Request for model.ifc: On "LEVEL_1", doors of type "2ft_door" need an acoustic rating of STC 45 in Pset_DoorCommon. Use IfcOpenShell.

First a look at what the model holds.

```python
import ifcopenshell
import ifcopenshell.util.element

model = ifcopenshell.open("model.ifc")
print(model.schema)
storey = next(s for s in model.by_type("IfcBuildingStorey") if s.Name == "LEVEL_1")
doors = [e for e in ifcopenshell.util.element.get_decomposition(storey) if e.is_a("IfcDoor")]
seen = {}
for e in doors:
    element_type = ifcopenshell.util.element.get_type(e)
    key = (element_type.Name if element_type != e and element_type else None, ifcopenshell.util.element.get_pset(e, "Pset_DoorCommon", "AcousticRating"))
    seen[key] = seen.get(key, 0) + 1
for (name, value), count in sorted(seen.items(), key=str):
    print(count, "x", name, "|", value)
```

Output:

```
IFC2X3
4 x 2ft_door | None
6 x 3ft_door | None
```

```python
import ifcopenshell
import ifcopenshell.api.pset
import ifcopenshell.util.element

model = ifcopenshell.open("model.ifc")

storey = next(s for s in model.by_type("IfcBuildingStorey") if s.Name == "LEVEL_1")
doors = [e for e in ifcopenshell.util.element.get_decomposition(storey) if e.is_a("IfcDoor")]

count = 0
for e in doors:
    element_type = ifcopenshell.util.element.get_type(e)
    if element_type in (None, e) or element_type.Name != "2ft_door":
        continue
    # add_pset returns the element's existing set when there is one.
    pset = ifcopenshell.api.pset.add_pset(model, product=e, name="Pset_DoorCommon")
    ifcopenshell.api.pset.edit_pset(model, pset=pset, properties={"AcousticRating": "STC 45"})
    count += 1

print(count, "doors updated")

model.write("model-out.ifc")
```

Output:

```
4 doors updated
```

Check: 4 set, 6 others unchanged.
